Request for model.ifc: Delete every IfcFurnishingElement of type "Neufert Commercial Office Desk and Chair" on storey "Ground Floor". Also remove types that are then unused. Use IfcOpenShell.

First a look at what the model holds.

```python
import ifcopenshell
import ifcopenshell.util.element

model = ifcopenshell.open("model.ifc")
print(model.schema)
storey = next(s for s in model.by_type("IfcBuildingStorey") if s.Name == "Ground Floor")
furniture = [e for e in ifcopenshell.util.element.get_decomposition(storey) if e.is_a("IfcFurnishingElement")]
seen = {}
for e in furniture:
    element_type = ifcopenshell.util.element.get_type(e)
    name = element_type.Name if element_type not in (None, e) else None
    seen[name] = seen.get(name, 0) + 1
for name, count in sorted(seen.items(), key=str):
    print(count, "x", name)
```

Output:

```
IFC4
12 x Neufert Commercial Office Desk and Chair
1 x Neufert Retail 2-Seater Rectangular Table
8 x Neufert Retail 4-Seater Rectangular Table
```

```python
import ifcopenshell
import ifcopenshell.api.root
import ifcopenshell.util.element

model = ifcopenshell.open("model.ifc")

storey = next(s for s in model.by_type("IfcBuildingStorey") if s.Name == "Ground Floor")
furniture = [e for e in ifcopenshell.util.element.get_decomposition(storey) if e.is_a("IfcFurnishingElement")]
targets = [e for e in furniture if (t := ifcopenshell.util.element.get_type(e)) not in (None, e) and t.Name == "Neufert Commercial Office Desk and Chair"]
types = {ifcopenshell.util.element.get_type(e) for e in targets} - {None, *targets}

for e in targets:
    ifcopenshell.api.root.remove_product(model, product=e)
print(len(targets), "removed")

unused = [t for t in types if not ifcopenshell.util.element.get_types(t)]
for t in unused:
    ifcopenshell.api.root.remove_product(model, product=t)
print(len(unused), "unused types removed")

model.write("model_rev.ifc")
```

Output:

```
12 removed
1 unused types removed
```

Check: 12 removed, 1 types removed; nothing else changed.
